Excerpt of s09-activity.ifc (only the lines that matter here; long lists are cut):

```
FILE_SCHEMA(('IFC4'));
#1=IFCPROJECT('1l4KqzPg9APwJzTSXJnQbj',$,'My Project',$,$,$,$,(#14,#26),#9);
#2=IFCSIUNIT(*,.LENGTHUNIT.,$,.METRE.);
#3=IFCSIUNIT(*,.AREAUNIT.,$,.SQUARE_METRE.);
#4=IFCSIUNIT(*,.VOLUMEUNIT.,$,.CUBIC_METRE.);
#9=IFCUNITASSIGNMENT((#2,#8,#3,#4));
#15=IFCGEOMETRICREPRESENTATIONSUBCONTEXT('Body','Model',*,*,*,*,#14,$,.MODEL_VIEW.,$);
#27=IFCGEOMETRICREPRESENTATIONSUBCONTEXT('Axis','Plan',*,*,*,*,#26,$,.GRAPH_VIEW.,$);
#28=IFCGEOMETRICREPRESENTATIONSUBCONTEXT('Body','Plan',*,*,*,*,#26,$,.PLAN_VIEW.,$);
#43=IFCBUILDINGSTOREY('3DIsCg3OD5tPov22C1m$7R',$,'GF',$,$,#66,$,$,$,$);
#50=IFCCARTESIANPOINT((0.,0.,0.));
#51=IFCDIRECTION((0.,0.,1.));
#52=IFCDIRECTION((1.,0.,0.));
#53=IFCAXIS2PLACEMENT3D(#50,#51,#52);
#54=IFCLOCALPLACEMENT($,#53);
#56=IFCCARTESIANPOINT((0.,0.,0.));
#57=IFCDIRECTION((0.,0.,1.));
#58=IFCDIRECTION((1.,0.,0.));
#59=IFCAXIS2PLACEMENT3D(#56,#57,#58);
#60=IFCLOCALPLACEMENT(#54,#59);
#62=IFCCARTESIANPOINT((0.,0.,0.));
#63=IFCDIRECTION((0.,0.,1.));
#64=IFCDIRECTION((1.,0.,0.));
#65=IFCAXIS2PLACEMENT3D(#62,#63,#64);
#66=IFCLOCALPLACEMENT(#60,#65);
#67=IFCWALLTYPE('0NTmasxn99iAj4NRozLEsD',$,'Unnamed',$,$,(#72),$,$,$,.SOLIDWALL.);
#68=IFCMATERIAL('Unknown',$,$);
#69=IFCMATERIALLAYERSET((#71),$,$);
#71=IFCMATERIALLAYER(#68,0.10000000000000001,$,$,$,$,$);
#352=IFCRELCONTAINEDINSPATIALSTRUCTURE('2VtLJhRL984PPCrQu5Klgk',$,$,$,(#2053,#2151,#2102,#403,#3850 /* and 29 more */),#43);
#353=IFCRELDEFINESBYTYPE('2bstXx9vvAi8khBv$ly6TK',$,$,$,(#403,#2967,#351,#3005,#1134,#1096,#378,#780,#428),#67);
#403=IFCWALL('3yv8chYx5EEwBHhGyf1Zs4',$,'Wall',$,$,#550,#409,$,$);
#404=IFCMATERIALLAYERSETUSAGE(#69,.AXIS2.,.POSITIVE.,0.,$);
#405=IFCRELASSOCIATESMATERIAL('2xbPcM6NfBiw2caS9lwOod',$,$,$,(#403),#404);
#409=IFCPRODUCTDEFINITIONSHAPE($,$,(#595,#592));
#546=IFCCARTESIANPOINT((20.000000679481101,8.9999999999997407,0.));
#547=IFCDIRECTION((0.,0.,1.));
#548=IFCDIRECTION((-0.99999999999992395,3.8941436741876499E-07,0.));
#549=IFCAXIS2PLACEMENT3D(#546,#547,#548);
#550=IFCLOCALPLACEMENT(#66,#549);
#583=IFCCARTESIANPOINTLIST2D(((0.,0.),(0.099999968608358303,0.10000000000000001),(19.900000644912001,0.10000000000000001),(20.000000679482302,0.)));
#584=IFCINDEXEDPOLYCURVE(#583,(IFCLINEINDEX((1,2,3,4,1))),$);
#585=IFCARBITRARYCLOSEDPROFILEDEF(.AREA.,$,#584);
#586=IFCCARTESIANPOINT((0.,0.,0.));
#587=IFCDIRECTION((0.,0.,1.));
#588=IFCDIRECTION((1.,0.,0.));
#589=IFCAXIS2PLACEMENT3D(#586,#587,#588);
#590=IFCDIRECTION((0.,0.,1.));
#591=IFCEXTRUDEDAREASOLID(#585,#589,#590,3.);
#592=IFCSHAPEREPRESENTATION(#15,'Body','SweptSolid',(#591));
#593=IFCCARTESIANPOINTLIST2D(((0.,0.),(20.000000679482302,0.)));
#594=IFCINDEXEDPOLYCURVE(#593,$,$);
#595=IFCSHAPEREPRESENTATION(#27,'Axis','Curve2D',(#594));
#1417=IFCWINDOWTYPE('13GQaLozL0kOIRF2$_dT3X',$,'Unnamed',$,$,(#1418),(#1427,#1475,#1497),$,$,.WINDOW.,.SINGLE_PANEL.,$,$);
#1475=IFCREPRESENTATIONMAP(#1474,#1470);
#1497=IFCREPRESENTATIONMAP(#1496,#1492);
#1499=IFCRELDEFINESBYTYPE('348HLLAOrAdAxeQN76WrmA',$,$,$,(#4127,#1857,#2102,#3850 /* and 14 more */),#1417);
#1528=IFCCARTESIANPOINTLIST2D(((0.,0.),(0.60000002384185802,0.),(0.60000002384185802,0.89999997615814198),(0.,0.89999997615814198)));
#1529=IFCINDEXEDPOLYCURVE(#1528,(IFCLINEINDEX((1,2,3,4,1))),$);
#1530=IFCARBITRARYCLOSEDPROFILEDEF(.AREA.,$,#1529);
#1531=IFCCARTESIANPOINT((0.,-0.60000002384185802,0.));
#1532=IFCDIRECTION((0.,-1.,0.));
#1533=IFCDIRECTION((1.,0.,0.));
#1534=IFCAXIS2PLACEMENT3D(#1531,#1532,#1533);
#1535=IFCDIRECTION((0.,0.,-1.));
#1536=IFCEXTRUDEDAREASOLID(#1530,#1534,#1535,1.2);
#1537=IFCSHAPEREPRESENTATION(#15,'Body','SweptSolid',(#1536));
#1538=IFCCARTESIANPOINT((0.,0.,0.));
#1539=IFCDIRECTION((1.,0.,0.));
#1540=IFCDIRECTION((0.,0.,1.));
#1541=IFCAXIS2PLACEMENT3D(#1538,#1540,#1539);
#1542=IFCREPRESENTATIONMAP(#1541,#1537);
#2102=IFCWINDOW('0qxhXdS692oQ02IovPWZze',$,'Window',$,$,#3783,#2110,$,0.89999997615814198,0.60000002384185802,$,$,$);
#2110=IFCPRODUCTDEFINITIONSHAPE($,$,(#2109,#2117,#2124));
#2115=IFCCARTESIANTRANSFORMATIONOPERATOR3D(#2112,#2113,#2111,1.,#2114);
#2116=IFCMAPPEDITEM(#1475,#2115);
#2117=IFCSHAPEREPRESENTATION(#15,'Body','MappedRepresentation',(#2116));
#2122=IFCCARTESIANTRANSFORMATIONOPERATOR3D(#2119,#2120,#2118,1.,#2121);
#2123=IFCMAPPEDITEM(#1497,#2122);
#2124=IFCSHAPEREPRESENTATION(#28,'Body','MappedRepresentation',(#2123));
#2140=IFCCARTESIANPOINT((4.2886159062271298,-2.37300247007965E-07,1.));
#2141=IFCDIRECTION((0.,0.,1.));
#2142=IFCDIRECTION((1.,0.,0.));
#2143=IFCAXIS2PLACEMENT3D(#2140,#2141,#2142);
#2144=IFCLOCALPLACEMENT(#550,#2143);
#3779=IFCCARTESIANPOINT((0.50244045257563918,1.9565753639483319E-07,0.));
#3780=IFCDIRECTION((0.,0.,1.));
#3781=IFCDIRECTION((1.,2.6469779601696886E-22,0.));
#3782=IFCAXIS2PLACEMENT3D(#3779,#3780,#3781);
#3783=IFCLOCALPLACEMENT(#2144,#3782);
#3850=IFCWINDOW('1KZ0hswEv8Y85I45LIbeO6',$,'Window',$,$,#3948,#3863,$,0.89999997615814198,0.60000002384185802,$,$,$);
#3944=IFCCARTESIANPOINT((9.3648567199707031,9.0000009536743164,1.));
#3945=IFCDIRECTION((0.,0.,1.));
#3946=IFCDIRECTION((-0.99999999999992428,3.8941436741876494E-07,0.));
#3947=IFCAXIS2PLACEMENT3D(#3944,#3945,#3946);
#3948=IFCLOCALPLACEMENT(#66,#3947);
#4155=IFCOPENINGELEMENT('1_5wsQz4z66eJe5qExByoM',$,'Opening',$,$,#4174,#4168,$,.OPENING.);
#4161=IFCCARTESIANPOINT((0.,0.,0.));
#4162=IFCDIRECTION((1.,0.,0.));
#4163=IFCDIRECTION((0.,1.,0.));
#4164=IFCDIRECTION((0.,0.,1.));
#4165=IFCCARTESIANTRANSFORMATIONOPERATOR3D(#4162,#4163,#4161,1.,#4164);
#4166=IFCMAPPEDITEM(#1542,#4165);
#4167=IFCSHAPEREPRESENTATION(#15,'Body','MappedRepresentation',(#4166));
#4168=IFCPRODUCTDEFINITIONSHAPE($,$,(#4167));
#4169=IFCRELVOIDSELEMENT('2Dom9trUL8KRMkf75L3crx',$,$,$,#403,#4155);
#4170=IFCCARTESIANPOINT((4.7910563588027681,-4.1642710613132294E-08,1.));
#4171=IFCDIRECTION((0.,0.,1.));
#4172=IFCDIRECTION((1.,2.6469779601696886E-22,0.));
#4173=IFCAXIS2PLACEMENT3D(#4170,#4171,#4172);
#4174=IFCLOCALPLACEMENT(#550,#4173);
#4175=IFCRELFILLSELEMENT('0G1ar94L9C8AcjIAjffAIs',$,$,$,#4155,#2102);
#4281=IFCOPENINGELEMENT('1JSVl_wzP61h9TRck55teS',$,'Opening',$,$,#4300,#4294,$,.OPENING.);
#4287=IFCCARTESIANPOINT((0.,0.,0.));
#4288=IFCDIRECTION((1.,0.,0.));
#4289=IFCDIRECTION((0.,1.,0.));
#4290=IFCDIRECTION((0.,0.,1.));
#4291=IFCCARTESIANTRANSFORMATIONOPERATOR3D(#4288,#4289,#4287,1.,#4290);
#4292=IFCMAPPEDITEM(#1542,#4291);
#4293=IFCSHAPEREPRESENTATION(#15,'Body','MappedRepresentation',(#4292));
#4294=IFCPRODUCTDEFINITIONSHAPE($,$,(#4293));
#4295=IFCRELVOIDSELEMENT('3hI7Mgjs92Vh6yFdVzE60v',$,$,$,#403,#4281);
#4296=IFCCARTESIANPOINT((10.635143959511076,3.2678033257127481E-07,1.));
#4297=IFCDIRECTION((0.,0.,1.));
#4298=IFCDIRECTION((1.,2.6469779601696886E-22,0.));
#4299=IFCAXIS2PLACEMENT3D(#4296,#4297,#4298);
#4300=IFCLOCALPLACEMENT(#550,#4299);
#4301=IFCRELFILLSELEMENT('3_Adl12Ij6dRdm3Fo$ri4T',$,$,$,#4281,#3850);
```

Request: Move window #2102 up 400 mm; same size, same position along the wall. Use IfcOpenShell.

```python
import numpy as np
import ifcopenshell
import ifcopenshell.api.geometry
import ifcopenshell.util.placement
import ifcopenshell.util.unit

model = ifcopenshell.open("s09-activity.ifc")
unit_scale = ifcopenshell.util.unit.calculate_unit_scale(model)

window = model.by_guid("0qxhXdS692oQ02IovPWZze")
opening = window.FillsVoids[0].RelatingOpeningElement
dz = 0.4 / unit_scale

shift = np.array([0.0, 0.0, dz])
# The window is not placed relative to its opening, so move both.
for product in (opening, window):
    matrix = ifcopenshell.util.placement.get_local_placement(product.ObjectPlacement)
    matrix[:3, 3] += shift
    ifcopenshell.api.geometry.edit_object_placement(model, product=product, matrix=matrix, is_si=False)

print(f"moved by {dz * unit_scale:+.3f} m")

model.write("s09-activity_rev.ifc")
```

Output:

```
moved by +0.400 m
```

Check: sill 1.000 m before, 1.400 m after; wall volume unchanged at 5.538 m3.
